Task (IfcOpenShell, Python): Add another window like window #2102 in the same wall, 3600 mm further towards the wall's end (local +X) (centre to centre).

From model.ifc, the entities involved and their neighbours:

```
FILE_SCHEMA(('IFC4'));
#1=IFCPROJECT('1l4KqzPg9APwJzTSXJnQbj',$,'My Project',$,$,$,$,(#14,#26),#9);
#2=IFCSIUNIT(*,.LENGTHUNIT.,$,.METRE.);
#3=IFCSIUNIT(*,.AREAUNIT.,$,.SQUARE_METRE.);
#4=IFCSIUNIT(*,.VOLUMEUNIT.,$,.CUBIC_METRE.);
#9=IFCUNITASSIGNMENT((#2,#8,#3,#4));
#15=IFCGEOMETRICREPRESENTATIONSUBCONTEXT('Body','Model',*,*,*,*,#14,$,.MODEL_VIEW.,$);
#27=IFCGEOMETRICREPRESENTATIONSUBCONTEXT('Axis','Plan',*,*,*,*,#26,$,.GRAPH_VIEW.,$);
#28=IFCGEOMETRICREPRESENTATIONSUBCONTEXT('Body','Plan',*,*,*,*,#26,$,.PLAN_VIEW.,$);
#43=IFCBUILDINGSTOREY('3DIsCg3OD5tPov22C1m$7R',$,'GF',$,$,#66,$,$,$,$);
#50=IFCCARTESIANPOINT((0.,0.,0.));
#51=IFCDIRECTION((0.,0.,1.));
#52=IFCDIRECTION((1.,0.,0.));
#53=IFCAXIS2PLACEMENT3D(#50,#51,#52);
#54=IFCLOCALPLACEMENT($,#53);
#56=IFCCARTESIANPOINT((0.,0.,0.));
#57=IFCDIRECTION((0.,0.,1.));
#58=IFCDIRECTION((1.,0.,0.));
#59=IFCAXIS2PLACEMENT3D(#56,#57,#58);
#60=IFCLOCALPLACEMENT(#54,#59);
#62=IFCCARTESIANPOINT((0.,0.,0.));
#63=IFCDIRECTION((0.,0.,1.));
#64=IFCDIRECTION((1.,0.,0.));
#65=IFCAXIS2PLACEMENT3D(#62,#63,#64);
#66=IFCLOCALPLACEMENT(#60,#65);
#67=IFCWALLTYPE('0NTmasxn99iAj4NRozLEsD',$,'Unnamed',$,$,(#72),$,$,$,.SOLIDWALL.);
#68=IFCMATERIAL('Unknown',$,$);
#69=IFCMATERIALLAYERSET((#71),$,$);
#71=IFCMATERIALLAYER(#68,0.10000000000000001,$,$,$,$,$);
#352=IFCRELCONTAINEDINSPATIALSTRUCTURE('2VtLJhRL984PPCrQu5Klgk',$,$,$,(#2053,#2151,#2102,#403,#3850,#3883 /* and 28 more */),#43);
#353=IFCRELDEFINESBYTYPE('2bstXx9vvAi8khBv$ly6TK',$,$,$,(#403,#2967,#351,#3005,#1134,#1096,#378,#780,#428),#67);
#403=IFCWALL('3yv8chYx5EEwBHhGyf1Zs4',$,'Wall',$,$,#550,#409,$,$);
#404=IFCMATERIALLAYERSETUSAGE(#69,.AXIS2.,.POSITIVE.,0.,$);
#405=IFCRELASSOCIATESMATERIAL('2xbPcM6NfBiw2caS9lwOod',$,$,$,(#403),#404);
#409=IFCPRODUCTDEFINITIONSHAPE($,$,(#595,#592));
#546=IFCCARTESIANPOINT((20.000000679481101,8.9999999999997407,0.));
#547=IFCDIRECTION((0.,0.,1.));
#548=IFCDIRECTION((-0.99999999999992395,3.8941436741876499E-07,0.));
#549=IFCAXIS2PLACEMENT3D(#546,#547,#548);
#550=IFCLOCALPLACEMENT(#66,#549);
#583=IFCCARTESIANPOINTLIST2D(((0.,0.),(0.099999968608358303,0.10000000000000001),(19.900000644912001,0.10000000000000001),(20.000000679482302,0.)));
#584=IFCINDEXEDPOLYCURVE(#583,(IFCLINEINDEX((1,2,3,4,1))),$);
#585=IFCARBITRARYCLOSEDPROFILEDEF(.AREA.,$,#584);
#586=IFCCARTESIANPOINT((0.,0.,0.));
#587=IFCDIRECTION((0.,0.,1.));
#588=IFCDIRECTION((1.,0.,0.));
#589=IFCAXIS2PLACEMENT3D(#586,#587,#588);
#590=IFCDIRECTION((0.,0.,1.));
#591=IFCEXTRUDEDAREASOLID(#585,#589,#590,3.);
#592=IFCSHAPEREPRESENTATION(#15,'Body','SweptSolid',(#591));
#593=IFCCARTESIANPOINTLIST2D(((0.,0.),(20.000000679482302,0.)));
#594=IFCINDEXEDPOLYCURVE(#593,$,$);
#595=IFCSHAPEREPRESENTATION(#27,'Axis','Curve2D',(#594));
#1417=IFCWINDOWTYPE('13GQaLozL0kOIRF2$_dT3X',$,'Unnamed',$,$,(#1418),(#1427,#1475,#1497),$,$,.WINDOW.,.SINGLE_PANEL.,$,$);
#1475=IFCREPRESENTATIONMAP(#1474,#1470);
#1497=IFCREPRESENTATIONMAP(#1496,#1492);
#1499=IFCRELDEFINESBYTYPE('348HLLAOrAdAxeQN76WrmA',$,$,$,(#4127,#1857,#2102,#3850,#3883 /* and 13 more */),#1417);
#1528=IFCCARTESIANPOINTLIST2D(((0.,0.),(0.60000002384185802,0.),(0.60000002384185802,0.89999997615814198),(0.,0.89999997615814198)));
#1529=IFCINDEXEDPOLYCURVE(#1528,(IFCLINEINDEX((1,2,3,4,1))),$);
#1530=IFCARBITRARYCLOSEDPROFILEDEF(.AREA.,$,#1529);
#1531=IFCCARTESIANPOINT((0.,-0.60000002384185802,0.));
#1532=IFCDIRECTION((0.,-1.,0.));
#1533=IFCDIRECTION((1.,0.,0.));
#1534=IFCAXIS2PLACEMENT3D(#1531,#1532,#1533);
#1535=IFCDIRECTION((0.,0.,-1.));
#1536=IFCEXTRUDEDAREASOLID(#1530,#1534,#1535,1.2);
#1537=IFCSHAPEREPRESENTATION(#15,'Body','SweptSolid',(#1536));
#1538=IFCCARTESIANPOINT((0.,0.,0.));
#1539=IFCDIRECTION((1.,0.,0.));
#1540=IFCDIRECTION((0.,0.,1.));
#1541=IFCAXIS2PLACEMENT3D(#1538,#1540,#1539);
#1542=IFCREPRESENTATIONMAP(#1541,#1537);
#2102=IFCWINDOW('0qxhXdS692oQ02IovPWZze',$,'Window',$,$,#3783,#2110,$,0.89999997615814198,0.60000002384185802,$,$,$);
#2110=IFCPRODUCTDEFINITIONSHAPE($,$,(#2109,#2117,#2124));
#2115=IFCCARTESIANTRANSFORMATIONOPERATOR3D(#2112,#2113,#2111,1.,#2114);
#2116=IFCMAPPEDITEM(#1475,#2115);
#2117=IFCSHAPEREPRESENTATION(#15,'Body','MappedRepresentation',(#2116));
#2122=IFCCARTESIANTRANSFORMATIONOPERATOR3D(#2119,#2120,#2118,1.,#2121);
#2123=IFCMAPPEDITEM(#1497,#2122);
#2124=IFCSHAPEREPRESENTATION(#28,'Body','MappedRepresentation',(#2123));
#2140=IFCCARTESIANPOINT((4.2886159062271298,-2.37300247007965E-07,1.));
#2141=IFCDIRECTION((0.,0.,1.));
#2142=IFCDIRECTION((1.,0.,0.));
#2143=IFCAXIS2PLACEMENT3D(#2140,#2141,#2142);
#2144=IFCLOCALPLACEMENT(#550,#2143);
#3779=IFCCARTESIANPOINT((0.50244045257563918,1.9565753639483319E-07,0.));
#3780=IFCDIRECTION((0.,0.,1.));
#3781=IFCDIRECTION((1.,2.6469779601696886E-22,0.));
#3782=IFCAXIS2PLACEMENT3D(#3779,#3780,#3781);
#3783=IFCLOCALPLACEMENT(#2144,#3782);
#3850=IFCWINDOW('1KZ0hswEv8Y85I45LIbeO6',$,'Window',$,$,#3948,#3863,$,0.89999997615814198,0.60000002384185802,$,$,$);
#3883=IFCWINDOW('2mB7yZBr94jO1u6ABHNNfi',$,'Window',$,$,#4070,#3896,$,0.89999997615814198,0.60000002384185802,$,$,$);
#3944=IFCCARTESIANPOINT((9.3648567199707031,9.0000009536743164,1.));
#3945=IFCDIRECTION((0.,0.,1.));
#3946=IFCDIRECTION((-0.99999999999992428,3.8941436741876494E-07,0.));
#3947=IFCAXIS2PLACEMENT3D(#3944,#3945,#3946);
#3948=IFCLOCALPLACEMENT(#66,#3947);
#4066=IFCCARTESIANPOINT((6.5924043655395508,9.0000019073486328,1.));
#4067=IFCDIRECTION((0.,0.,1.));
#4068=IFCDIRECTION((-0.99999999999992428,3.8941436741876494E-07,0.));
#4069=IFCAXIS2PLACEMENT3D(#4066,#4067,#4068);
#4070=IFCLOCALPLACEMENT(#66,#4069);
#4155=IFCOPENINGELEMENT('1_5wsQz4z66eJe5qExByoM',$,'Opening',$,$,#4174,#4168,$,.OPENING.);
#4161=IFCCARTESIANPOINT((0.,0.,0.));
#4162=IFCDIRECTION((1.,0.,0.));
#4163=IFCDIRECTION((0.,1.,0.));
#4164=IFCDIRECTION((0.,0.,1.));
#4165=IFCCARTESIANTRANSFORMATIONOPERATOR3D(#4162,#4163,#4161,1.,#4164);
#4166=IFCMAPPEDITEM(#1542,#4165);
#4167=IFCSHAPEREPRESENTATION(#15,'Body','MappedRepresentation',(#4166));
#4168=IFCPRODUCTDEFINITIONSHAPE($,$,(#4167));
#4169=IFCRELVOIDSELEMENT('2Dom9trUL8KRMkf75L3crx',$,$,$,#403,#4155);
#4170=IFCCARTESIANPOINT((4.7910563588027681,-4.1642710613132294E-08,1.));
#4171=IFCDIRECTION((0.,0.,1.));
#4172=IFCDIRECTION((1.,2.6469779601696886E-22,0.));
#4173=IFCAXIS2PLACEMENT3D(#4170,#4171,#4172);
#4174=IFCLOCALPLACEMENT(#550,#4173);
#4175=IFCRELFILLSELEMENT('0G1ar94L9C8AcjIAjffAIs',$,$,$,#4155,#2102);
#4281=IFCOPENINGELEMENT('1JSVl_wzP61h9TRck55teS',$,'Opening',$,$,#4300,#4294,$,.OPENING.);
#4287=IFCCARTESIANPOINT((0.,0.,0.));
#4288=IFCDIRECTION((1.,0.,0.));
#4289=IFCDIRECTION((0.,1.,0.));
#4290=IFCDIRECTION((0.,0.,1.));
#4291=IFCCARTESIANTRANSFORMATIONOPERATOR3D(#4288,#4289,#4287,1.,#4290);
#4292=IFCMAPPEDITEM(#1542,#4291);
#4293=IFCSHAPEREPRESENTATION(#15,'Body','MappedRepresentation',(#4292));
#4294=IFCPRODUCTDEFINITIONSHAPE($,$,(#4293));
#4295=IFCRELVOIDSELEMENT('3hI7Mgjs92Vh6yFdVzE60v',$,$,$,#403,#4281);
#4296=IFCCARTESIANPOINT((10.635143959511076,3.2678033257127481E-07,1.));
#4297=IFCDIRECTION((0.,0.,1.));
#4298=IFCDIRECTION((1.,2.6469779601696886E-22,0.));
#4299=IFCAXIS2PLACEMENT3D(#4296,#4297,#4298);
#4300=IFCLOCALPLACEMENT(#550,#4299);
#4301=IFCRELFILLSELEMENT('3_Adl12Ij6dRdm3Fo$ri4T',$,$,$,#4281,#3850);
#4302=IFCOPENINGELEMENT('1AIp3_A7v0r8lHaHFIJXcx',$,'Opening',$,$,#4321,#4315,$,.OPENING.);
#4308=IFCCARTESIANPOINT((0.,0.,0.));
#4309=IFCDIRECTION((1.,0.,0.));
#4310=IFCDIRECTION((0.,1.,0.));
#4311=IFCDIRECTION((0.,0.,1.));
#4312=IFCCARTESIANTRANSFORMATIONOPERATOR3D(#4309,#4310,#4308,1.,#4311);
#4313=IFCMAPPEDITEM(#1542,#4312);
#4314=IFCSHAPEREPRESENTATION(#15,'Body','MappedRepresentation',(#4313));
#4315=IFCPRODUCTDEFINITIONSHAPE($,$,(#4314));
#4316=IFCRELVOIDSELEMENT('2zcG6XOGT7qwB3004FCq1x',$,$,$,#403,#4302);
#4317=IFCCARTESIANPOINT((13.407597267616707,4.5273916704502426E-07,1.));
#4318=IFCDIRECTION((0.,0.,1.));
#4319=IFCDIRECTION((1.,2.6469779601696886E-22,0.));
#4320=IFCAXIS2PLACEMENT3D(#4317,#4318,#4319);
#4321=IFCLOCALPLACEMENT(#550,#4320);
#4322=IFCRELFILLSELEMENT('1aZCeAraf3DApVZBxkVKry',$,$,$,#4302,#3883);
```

```python
import ifcopenshell
import ifcopenshell.api.feature
import ifcopenshell.api.geometry
import ifcopenshell.api.root
import ifcopenshell.geom
import ifcopenshell.util.element
import ifcopenshell.util.placement
import ifcopenshell.util.shape

model = ifcopenshell.open("model.ifc")
settings = ifcopenshell.geom.settings()


def volume(element):
    """Net volume in cubic metres, openings subtracted."""
    shape = ifcopenshell.geom.create_shape(settings, element)
    return ifcopenshell.util.shape.get_volume(shape.geometry)


window = model.by_guid("0qxhXdS692oQ02IovPWZze")
opening = window.FillsVoids[0].RelatingOpeningElement
wall = opening.VoidsElements[0].RelatingBuildingElement
before = volume(wall)
shift = ifcopenshell.util.placement.get_local_placement(wall.ObjectPlacement)[:3, 0] * 3.6

# copy_class copies the void relationship, type, container and properties, but no geometry.
new_opening = ifcopenshell.api.root.copy_class(model, product=opening)
new_opening.Representation = ifcopenshell.util.element.copy_deep(
    model, opening.Representation, exclude=["IfcGeometricRepresentationContext", "IfcRepresentationMap"]
)
new_window = ifcopenshell.api.root.copy_class(model, product=window)
new_window.Representation = ifcopenshell.util.element.copy_deep(
    model, window.Representation, exclude=["IfcGeometricRepresentationContext", "IfcRepresentationMap"]
)
ifcopenshell.api.feature.add_filling(model, opening=new_opening, element=new_window)

for old, new in ((opening, new_opening), (window, new_window)):
    matrix = ifcopenshell.util.placement.get_local_placement(old.ObjectPlacement)
    matrix[:3, 3] += shift
    ifcopenshell.api.geometry.edit_object_placement(model, product=new, matrix=matrix, is_si=False)

after = volume(wall)

print(f"wall volume {before:.3f} -> {after:.3f} m3")

model.write("model_v2.ifc")
```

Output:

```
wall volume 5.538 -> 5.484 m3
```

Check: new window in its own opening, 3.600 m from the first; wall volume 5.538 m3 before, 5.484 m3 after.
